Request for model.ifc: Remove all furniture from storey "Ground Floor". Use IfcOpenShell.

First a look at what the model holds.

```python
import ifcopenshell
import ifcopenshell.util.element

model = ifcopenshell.open("model.ifc")
print(model.schema)
storey = next(s for s in model.by_type("IfcBuildingStorey") if s.Name == "Ground Floor")
furniture = [e for e in ifcopenshell.util.element.get_decomposition(storey) if e.is_a("IfcFurnishingElement")]
seen = {}
for e in furniture:
    element_type = ifcopenshell.util.element.get_type(e)
    name = element_type.Name if element_type not in (None, e) else None
    seen[name] = seen.get(name, 0) + 1
for name, count in sorted(seen.items(), key=str):
    print(count, "x", name)
```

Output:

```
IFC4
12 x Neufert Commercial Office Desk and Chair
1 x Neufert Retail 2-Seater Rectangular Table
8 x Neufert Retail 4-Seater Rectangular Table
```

```python
import ifcopenshell
import ifcopenshell.api.root
import ifcopenshell.util.element

model = ifcopenshell.open("model.ifc")

storey = next(s for s in model.by_type("IfcBuildingStorey") if s.Name == "Ground Floor")
furniture = [e for e in ifcopenshell.util.element.get_decomposition(storey) if e.is_a("IfcFurnishingElement")]

for e in furniture:
    ifcopenshell.api.root.remove_product(model, product=e)
print(len(furniture), "removed")

model.write("model_edited.ifc")
```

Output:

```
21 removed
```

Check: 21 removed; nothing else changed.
